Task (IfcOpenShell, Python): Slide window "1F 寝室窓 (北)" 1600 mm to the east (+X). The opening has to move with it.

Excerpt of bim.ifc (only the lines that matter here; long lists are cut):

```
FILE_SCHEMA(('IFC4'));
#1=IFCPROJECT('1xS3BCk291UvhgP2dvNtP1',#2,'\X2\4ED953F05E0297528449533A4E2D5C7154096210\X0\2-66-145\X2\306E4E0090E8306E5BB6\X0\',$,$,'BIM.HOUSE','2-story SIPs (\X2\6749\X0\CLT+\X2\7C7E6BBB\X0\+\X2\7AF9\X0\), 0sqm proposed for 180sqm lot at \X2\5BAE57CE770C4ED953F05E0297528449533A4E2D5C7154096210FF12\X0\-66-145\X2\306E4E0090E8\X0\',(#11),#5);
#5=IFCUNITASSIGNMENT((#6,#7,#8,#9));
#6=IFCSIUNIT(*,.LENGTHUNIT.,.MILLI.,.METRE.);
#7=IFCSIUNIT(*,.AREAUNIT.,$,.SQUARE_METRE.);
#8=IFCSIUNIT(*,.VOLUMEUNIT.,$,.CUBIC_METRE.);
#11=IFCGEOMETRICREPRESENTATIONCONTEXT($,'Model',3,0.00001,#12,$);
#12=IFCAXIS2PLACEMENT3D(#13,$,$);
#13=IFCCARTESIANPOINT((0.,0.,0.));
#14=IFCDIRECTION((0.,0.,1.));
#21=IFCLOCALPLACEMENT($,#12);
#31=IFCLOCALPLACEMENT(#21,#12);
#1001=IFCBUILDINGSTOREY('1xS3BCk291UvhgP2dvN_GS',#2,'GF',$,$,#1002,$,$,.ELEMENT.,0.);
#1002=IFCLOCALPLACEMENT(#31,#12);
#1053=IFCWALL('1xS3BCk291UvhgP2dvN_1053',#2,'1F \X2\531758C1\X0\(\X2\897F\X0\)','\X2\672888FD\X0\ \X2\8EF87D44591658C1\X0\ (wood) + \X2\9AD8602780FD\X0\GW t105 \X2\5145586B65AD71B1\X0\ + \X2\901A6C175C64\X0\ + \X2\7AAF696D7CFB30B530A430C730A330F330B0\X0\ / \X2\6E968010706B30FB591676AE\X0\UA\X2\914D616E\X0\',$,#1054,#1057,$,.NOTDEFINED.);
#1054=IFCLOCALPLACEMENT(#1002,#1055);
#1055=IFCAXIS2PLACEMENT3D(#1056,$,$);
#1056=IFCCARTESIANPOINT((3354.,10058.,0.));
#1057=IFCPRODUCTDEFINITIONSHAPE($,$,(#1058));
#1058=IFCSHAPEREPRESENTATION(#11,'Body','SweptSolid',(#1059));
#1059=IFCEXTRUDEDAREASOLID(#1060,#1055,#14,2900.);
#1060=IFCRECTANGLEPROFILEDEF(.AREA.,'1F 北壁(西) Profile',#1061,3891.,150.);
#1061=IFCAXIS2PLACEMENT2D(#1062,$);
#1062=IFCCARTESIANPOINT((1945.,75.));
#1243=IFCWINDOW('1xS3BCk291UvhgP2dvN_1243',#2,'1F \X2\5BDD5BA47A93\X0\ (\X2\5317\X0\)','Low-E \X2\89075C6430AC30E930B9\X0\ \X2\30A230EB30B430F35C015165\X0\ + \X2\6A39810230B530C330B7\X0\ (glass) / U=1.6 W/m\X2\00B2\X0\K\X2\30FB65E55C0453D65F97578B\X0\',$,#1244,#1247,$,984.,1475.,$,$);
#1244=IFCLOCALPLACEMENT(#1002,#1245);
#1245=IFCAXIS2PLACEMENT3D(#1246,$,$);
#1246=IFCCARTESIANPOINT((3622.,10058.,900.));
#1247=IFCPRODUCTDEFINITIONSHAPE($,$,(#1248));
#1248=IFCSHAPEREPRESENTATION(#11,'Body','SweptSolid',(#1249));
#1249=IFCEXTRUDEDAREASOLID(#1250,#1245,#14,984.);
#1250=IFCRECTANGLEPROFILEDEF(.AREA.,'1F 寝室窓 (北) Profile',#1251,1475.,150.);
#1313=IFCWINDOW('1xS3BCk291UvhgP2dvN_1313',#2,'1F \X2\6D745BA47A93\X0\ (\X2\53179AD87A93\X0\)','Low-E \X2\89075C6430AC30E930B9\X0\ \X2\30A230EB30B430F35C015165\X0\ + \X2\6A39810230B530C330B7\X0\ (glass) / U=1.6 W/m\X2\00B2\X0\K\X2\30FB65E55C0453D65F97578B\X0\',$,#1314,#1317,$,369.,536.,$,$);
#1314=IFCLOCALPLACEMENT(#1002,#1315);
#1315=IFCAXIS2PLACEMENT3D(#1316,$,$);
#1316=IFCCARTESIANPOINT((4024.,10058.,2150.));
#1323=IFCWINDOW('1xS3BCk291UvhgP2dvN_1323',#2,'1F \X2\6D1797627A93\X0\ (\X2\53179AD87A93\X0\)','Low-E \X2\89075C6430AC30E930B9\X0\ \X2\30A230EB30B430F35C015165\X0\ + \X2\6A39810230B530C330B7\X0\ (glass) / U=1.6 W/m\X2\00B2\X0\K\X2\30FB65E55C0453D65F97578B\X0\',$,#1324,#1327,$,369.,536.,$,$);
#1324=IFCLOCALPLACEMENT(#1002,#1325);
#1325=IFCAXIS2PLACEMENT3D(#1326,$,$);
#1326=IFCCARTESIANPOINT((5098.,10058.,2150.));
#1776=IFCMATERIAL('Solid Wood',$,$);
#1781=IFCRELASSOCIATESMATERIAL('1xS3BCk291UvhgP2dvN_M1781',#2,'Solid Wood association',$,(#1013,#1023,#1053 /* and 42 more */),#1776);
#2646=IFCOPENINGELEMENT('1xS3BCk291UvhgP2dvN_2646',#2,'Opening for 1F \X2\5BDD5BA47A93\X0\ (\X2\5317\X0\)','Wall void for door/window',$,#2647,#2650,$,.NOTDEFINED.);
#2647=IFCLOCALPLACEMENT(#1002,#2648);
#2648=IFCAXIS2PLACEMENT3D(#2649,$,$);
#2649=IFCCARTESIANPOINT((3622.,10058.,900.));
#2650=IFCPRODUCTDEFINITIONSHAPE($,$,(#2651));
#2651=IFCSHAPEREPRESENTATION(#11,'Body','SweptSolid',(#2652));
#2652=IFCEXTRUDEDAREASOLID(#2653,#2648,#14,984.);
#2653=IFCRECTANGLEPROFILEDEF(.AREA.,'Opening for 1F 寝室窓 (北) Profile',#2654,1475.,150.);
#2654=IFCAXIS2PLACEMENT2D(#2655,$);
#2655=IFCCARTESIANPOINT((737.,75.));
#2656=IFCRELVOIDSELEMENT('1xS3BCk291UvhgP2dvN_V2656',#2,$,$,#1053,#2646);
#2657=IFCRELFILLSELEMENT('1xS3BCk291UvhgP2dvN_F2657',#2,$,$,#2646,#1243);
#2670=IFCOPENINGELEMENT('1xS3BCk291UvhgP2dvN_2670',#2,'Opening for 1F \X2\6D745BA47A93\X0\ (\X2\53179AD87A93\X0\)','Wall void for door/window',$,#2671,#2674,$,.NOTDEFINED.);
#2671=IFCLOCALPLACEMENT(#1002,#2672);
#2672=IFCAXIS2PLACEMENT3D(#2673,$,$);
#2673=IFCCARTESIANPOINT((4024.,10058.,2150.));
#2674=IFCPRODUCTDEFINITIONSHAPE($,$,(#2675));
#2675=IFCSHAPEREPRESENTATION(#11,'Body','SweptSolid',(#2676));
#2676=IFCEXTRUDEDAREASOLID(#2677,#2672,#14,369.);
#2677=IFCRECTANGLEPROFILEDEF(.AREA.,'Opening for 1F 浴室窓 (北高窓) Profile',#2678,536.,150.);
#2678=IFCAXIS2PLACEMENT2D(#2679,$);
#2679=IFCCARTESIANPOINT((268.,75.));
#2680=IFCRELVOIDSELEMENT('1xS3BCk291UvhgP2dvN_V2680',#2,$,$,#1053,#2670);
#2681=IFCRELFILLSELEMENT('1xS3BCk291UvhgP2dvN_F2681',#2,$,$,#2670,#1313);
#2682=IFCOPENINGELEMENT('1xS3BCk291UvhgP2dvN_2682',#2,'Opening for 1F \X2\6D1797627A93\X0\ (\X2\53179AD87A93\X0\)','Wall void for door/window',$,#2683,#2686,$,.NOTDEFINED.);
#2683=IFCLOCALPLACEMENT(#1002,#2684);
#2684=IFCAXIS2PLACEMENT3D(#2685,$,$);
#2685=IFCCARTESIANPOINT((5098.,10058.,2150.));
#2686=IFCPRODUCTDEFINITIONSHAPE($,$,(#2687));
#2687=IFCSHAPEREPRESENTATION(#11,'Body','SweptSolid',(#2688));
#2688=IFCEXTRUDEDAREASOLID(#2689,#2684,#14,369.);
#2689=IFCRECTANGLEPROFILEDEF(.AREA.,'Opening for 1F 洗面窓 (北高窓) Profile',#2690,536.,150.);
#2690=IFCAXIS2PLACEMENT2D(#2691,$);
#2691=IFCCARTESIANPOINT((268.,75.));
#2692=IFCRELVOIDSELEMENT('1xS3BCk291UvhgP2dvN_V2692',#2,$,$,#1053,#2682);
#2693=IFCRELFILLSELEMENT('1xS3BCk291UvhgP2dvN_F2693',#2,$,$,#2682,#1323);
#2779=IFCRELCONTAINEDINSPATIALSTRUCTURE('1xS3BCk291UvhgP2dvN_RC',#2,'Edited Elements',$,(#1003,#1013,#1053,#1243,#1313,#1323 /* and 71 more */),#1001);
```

```python
import ifcopenshell
import ifcopenshell.api.geometry
import ifcopenshell.util.placement
import ifcopenshell.util.unit

model = ifcopenshell.open("bim.ifc")
unit_scale = ifcopenshell.util.unit.calculate_unit_scale(model)

window = model.by_guid("1xS3BCk291UvhgP2dvN_1243")
opening = window.FillsVoids[0].RelatingOpeningElement
wall = opening.VoidsElements[0].RelatingBuildingElement

wall_matrix = ifcopenshell.util.placement.get_local_placement(wall.ObjectPlacement)
shift = wall_matrix[:3, 0] * 1.6 / unit_scale
before = ifcopenshell.util.placement.get_local_placement(window.ObjectPlacement)[:3, 3].copy()

# The window is not placed relative to its opening, so move both.
for product in (opening, window):
    matrix = ifcopenshell.util.placement.get_local_placement(product.ObjectPlacement)
    matrix[:3, 3] += shift
    ifcopenshell.api.geometry.edit_object_placement(model, product=product, matrix=matrix, is_si=False)

after = ifcopenshell.util.placement.get_local_placement(window.ObjectPlacement)[:3, 3]
print("window moved by", (after - before).round(3) + 0.0)

model.write("bim-out.ifc")
```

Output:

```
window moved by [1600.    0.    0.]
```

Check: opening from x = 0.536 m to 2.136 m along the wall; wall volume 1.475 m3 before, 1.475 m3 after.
